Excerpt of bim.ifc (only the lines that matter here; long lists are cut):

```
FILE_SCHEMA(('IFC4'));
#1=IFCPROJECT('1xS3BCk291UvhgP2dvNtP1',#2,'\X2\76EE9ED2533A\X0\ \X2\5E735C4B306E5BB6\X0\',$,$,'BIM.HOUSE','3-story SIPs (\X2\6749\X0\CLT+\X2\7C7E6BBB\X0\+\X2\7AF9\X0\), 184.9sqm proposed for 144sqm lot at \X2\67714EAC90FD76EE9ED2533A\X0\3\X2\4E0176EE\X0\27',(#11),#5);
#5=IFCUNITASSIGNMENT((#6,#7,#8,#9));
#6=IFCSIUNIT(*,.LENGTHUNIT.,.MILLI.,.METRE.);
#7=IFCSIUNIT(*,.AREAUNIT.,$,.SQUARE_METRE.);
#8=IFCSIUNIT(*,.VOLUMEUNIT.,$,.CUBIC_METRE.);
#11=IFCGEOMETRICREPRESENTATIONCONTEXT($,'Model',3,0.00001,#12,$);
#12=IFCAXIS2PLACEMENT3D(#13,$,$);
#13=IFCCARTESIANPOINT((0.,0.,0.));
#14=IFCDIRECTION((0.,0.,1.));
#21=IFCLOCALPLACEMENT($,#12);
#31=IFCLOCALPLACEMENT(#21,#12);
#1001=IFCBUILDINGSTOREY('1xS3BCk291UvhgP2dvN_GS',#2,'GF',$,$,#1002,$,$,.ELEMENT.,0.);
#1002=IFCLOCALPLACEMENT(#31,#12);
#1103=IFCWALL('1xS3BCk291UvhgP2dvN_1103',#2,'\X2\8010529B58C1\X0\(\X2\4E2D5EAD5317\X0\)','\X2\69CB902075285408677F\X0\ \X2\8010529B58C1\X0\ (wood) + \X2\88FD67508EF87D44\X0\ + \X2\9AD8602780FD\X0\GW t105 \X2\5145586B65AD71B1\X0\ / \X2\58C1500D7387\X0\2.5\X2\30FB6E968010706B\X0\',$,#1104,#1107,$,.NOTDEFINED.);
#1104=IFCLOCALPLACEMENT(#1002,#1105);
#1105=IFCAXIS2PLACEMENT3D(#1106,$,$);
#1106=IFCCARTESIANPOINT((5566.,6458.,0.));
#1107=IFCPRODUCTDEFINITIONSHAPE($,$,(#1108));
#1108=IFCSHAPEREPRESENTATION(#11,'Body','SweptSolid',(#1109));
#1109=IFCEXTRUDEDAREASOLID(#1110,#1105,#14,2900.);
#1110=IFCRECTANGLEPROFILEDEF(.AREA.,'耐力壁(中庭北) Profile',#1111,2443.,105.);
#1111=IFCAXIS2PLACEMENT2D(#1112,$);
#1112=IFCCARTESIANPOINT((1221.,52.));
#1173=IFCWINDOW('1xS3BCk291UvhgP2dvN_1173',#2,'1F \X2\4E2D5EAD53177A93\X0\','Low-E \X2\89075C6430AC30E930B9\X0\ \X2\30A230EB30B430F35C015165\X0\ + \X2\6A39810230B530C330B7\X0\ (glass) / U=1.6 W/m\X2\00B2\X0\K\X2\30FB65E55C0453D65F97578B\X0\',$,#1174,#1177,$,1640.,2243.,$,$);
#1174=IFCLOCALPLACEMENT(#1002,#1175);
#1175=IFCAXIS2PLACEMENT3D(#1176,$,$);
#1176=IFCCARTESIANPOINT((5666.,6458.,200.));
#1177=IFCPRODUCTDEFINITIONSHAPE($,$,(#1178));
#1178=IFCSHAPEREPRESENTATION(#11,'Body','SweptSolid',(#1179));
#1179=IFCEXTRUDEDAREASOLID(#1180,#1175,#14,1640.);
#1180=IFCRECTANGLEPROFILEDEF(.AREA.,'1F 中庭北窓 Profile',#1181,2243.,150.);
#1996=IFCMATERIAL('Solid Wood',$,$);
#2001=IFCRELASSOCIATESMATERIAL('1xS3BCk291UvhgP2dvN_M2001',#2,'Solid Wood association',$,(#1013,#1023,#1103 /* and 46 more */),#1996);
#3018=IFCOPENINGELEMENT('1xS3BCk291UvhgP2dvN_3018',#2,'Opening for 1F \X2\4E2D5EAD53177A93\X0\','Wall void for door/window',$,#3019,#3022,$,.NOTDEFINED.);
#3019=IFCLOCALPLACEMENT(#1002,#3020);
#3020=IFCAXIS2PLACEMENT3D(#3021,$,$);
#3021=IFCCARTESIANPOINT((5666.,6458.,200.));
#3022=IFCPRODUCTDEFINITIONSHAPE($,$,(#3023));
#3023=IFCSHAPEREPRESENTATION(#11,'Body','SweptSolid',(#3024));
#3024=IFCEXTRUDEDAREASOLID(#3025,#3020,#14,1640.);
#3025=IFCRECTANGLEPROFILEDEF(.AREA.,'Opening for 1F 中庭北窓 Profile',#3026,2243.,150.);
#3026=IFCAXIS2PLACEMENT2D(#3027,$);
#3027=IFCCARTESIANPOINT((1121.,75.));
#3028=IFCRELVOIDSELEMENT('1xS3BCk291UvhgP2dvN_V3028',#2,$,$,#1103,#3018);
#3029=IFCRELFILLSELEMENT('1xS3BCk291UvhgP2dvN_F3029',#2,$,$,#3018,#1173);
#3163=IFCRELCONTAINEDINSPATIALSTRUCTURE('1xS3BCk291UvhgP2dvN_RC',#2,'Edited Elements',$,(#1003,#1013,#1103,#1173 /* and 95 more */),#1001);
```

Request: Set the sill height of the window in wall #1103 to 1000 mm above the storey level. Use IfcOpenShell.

```python
import numpy as np
import ifcopenshell
import ifcopenshell.api.geometry
import ifcopenshell.geom
import ifcopenshell.util.element
import ifcopenshell.util.placement
import ifcopenshell.util.shape
import ifcopenshell.util.unit

model = ifcopenshell.open("bim.ifc")
unit_scale = ifcopenshell.util.unit.calculate_unit_scale(model)

window = model.by_guid("1xS3BCk291UvhgP2dvN_1173")
opening = window.FillsVoids[0].RelatingOpeningElement
storey = ifcopenshell.util.element.get_container(window, ifc_class="IfcBuildingStorey")
level = ifcopenshell.util.placement.get_local_placement(storey.ObjectPlacement)[2, 3]

# The opening's origin need not be at the sill, so measure its lowest point.
shape = ifcopenshell.geom.create_shape(ifcopenshell.geom.settings(), opening)
bottom = ifcopenshell.util.shape.get_shape_bottom_elevation(shape, shape.geometry) / unit_scale
dz = level + 1 / unit_scale - bottom

shift = np.array([0.0, 0.0, dz])
# The window is not placed relative to its opening, so move both.
for product in (opening, window):
    matrix = ifcopenshell.util.placement.get_local_placement(product.ObjectPlacement)
    matrix[:3, 3] += shift
    ifcopenshell.api.geometry.edit_object_placement(model, product=product, matrix=matrix, is_si=False)

print(f"moved by {dz * unit_scale:+.3f} m")

model.write("bim-out.ifc")
```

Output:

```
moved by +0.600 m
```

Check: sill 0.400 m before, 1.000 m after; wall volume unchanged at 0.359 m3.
